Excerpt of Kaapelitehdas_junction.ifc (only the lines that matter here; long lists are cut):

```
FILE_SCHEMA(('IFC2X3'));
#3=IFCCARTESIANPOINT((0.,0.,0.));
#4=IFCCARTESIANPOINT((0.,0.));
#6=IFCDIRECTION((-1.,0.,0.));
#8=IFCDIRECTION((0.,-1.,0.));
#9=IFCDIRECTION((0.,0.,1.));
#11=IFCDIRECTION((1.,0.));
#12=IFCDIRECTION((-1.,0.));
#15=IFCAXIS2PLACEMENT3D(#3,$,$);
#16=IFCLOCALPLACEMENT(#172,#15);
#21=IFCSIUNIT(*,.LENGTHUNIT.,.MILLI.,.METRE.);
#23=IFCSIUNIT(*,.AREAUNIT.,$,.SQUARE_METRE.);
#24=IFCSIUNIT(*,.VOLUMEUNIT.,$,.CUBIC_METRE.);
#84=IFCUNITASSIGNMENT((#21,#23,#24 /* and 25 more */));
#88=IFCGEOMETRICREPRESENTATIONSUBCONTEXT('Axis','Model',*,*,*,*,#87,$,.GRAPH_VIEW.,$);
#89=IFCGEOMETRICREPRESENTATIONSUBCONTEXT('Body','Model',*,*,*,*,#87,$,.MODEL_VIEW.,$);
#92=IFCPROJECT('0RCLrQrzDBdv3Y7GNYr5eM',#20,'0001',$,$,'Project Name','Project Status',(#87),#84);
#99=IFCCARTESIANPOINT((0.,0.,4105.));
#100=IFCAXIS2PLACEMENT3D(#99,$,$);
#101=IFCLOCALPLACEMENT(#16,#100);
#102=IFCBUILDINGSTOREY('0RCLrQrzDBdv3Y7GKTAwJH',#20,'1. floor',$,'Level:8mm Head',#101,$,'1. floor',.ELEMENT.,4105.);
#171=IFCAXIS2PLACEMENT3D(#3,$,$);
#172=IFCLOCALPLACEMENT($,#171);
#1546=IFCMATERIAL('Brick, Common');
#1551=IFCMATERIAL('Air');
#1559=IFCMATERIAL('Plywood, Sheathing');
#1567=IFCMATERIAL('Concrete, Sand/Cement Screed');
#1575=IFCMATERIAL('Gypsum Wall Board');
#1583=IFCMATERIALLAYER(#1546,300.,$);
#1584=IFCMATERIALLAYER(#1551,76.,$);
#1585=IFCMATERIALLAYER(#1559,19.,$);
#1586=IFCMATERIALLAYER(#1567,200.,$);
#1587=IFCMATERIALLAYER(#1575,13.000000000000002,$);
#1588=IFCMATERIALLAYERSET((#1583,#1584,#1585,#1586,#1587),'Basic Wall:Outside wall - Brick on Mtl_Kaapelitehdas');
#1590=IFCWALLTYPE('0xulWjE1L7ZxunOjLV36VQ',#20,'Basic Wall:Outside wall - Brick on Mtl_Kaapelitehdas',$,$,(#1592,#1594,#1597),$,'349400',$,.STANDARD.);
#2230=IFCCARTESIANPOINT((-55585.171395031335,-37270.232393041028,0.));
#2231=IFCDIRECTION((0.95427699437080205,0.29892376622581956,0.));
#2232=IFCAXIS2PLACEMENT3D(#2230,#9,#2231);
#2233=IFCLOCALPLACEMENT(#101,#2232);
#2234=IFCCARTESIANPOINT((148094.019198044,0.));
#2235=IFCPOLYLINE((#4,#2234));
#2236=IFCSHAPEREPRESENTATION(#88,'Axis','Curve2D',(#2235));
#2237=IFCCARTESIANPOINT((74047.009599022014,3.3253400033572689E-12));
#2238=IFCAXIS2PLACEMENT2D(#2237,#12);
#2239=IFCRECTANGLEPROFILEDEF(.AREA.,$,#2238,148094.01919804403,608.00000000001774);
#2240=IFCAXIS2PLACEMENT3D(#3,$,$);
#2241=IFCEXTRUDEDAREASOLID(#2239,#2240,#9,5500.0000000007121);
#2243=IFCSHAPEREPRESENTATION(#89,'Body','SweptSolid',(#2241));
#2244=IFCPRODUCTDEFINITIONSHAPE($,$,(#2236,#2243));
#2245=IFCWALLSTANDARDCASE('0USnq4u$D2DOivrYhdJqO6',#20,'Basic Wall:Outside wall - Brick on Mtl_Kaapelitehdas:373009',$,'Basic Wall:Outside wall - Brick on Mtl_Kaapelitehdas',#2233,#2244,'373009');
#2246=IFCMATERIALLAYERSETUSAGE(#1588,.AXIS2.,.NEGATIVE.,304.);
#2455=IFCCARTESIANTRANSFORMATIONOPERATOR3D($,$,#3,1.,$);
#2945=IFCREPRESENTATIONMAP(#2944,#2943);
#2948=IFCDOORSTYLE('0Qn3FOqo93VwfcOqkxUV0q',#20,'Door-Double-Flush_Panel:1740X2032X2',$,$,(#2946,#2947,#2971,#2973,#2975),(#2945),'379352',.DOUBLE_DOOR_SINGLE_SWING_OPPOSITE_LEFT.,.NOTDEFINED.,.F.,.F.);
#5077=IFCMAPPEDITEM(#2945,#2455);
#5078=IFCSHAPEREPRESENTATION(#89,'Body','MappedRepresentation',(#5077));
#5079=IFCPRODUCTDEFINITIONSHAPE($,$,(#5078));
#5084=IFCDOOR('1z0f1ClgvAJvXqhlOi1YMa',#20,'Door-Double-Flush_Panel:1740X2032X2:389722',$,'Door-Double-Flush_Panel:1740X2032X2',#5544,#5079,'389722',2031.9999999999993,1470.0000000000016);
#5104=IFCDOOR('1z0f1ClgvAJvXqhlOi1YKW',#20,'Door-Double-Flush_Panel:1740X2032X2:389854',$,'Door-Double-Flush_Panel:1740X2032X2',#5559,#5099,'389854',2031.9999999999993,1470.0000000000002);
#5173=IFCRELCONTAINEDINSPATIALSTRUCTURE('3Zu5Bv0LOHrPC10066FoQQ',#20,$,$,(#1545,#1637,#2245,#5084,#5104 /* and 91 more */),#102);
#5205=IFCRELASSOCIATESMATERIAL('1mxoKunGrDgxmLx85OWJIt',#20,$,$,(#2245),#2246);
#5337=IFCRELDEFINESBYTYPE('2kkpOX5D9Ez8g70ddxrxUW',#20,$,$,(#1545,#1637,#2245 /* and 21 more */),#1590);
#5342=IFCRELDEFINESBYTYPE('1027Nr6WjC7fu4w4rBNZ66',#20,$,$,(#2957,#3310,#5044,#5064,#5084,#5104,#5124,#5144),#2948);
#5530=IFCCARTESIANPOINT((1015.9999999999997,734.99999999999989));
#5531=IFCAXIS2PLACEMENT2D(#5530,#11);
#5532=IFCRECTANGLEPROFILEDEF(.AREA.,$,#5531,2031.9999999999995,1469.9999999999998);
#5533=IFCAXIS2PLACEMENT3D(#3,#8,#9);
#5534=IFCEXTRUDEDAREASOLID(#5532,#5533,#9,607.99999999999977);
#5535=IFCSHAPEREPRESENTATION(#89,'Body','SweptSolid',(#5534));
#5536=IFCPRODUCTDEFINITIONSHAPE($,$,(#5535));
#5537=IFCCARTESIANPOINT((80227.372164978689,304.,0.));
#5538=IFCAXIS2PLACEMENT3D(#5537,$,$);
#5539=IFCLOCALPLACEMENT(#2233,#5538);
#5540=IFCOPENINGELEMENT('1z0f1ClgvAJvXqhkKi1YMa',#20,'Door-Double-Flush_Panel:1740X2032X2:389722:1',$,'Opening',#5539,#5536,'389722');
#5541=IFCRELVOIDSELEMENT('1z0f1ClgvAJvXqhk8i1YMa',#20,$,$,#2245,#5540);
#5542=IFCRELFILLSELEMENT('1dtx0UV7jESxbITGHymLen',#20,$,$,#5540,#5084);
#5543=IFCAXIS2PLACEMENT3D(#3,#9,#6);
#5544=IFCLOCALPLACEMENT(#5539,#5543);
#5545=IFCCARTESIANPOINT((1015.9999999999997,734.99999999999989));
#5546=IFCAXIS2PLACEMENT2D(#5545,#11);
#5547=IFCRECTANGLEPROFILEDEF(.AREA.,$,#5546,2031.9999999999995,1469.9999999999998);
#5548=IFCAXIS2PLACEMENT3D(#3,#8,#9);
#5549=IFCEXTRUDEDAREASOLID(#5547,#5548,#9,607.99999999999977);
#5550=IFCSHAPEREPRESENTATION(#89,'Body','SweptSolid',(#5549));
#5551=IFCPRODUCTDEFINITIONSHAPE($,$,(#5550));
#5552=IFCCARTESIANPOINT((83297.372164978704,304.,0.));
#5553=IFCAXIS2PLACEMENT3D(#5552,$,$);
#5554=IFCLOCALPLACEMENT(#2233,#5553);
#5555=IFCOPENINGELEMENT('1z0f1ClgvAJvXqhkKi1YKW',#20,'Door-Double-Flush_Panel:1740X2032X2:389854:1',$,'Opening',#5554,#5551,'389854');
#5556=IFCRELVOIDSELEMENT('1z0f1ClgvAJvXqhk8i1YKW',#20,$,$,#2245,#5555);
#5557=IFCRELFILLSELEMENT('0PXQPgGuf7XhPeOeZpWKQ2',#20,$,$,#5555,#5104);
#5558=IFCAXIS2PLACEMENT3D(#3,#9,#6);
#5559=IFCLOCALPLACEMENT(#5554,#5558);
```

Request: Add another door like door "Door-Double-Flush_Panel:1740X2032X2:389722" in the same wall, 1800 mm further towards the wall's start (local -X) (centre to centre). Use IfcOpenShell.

```python
import ifcopenshell
import ifcopenshell.api.feature
import ifcopenshell.api.geometry
import ifcopenshell.api.root
import ifcopenshell.geom
import ifcopenshell.util.element
import ifcopenshell.util.placement
import ifcopenshell.util.shape

model = ifcopenshell.open("Kaapelitehdas_junction.ifc")
settings = ifcopenshell.geom.settings()


def volume(element):
    """Net volume in cubic metres, openings subtracted."""
    shape = ifcopenshell.geom.create_shape(settings, element)
    return ifcopenshell.util.shape.get_volume(shape.geometry)


def reuse_history(source, copy):
    """copy_class also copies each property set's owner history, people and application; keep the originals."""
    for rel in copy.IsDefinedBy:
        if rel.is_a("IfcRelDefinesByProperties") and (history := rel.RelatingPropertyDefinition.OwnerHistory):
            rel.RelatingPropertyDefinition.OwnerHistory = source.OwnerHistory
            ifcopenshell.util.element.remove_deep2(model, history)


door = model.by_guid("1z0f1ClgvAJvXqhlOi1YMa")
opening = door.FillsVoids[0].RelatingOpeningElement
wall = opening.VoidsElements[0].RelatingBuildingElement
before = volume(wall)
shift = ifcopenshell.util.placement.get_local_placement(wall.ObjectPlacement)[:3, 0] * -1800.0

# copy_class copies the void relationship, type, container and properties, but no geometry.
new_opening = ifcopenshell.api.root.copy_class(model, product=opening)
new_opening.Representation = ifcopenshell.util.element.copy_deep(
    model, opening.Representation, exclude=["IfcGeometricRepresentationContext", "IfcRepresentationMap"]
)
new_opening.Name = "Door-Double-Flush_Panel:1740X2032X2"
new_opening.Tag = None
new_door = ifcopenshell.api.root.copy_class(model, product=door)
new_door.Representation = ifcopenshell.util.element.copy_deep(
    model, door.Representation, exclude=["IfcGeometricRepresentationContext", "IfcRepresentationMap"]
)
new_door.Name = "Door-Double-Flush_Panel:1740X2032X2"
new_door.Tag = None
reuse_history(door, new_door)
fills = ifcopenshell.api.feature.add_filling(model, opening=new_opening, element=new_door)
fills.OwnerHistory = new_door.OwnerHistory  # required in IFC2X3

for old, new in ((opening, new_opening), (door, new_door)):
    matrix = ifcopenshell.util.placement.get_local_placement(old.ObjectPlacement)
    matrix[:3, 3] += shift
    ifcopenshell.api.geometry.edit_object_placement(model, product=new, matrix=matrix, is_si=False)

after = volume(wall)

print(f"wall volume {before:.3f} -> {after:.3f} m3")

model.write("Kaapelitehdas_junction_updated.ifc")
```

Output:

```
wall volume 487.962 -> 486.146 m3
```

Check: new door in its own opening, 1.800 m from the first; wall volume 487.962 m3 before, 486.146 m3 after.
